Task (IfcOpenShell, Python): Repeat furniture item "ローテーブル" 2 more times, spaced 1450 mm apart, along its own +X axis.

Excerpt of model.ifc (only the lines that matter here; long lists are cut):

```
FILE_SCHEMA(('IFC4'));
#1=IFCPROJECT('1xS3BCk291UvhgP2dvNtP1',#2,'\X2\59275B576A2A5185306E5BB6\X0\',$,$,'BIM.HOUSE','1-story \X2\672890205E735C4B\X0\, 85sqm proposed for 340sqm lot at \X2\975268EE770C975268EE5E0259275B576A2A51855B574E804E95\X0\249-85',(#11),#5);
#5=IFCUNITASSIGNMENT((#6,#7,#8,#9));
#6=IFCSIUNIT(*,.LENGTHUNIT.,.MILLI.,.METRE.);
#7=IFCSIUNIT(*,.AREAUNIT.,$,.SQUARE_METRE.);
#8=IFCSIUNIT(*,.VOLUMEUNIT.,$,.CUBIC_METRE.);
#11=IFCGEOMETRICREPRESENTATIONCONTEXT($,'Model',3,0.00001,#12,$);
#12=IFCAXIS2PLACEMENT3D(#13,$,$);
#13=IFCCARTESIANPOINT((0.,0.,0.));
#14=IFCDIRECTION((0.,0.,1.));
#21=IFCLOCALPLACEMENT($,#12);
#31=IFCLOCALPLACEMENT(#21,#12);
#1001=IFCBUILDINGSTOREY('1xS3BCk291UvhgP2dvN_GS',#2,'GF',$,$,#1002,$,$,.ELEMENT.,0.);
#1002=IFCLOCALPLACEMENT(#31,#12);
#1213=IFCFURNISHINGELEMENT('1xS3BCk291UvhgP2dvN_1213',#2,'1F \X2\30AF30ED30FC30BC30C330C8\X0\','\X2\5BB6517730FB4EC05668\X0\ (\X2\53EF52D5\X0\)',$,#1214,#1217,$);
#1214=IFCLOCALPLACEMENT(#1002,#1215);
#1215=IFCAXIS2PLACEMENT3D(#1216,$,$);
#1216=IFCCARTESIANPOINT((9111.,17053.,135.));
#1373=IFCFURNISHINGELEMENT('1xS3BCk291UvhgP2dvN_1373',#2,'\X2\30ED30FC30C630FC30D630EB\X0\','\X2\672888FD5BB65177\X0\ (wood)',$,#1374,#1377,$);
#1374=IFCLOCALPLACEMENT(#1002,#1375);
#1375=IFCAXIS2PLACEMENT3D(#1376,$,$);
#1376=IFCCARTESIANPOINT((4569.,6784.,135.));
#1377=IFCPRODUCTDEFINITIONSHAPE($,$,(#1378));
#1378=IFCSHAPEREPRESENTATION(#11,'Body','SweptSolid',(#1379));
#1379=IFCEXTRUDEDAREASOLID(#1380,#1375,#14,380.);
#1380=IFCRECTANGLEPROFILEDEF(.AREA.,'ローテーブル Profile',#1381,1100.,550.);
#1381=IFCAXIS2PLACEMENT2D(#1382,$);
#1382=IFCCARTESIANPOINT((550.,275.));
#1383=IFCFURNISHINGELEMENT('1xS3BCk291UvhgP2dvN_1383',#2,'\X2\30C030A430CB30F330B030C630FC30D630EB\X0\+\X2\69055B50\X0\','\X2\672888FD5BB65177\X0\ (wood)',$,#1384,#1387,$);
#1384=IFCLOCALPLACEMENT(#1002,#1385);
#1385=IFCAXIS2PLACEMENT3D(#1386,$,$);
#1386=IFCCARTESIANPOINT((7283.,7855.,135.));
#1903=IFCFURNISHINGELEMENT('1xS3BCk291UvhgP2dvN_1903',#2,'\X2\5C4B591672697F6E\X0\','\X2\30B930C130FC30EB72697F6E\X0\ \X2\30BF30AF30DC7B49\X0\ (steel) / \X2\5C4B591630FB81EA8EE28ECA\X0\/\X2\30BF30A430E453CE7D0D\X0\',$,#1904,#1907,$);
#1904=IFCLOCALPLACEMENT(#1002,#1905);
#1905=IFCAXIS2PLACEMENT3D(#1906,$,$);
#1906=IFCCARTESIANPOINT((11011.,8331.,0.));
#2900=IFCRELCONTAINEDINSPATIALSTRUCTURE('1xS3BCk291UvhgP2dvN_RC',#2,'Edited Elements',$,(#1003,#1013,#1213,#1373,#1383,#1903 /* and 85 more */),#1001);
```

```python
import ifcopenshell
import ifcopenshell.api.geometry
import ifcopenshell.api.root
import ifcopenshell.util.element
import ifcopenshell.util.placement

model = ifcopenshell.open("model.ifc")


def reuse_history(source, copy):
    """copy_class also copies each property set's owner history, people and application; keep the originals."""
    for rel in copy.IsDefinedBy:
        if rel.is_a("IfcRelDefinesByProperties") and (history := rel.RelatingPropertyDefinition.OwnerHistory):
            rel.RelatingPropertyDefinition.OwnerHistory = source.OwnerHistory
            ifcopenshell.util.element.remove_deep2(model, history)


source = model.by_guid("1xS3BCk291UvhgP2dvN_1373")
base = ifcopenshell.util.placement.get_local_placement(source.ObjectPlacement)
step = base[:3, 0] * 1450.0

for i in range(1, 3):
    copy = ifcopenshell.api.root.copy_class(model, product=source)
    copy.Representation = ifcopenshell.util.element.copy_deep(
        model, source.Representation, exclude=["IfcGeometricRepresentationContext", "IfcRepresentationMap"]
    )
    reuse_history(source, copy)
    matrix = base.copy()
    matrix[:3, 3] += i * step
    print("added at", matrix[:3, 3].round(3) + 0.0)
    ifcopenshell.api.geometry.edit_object_placement(model, product=copy, matrix=matrix, is_si=False)

model.write("model_updated.ifc")
```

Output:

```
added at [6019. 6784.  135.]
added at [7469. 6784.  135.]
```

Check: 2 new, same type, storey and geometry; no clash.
